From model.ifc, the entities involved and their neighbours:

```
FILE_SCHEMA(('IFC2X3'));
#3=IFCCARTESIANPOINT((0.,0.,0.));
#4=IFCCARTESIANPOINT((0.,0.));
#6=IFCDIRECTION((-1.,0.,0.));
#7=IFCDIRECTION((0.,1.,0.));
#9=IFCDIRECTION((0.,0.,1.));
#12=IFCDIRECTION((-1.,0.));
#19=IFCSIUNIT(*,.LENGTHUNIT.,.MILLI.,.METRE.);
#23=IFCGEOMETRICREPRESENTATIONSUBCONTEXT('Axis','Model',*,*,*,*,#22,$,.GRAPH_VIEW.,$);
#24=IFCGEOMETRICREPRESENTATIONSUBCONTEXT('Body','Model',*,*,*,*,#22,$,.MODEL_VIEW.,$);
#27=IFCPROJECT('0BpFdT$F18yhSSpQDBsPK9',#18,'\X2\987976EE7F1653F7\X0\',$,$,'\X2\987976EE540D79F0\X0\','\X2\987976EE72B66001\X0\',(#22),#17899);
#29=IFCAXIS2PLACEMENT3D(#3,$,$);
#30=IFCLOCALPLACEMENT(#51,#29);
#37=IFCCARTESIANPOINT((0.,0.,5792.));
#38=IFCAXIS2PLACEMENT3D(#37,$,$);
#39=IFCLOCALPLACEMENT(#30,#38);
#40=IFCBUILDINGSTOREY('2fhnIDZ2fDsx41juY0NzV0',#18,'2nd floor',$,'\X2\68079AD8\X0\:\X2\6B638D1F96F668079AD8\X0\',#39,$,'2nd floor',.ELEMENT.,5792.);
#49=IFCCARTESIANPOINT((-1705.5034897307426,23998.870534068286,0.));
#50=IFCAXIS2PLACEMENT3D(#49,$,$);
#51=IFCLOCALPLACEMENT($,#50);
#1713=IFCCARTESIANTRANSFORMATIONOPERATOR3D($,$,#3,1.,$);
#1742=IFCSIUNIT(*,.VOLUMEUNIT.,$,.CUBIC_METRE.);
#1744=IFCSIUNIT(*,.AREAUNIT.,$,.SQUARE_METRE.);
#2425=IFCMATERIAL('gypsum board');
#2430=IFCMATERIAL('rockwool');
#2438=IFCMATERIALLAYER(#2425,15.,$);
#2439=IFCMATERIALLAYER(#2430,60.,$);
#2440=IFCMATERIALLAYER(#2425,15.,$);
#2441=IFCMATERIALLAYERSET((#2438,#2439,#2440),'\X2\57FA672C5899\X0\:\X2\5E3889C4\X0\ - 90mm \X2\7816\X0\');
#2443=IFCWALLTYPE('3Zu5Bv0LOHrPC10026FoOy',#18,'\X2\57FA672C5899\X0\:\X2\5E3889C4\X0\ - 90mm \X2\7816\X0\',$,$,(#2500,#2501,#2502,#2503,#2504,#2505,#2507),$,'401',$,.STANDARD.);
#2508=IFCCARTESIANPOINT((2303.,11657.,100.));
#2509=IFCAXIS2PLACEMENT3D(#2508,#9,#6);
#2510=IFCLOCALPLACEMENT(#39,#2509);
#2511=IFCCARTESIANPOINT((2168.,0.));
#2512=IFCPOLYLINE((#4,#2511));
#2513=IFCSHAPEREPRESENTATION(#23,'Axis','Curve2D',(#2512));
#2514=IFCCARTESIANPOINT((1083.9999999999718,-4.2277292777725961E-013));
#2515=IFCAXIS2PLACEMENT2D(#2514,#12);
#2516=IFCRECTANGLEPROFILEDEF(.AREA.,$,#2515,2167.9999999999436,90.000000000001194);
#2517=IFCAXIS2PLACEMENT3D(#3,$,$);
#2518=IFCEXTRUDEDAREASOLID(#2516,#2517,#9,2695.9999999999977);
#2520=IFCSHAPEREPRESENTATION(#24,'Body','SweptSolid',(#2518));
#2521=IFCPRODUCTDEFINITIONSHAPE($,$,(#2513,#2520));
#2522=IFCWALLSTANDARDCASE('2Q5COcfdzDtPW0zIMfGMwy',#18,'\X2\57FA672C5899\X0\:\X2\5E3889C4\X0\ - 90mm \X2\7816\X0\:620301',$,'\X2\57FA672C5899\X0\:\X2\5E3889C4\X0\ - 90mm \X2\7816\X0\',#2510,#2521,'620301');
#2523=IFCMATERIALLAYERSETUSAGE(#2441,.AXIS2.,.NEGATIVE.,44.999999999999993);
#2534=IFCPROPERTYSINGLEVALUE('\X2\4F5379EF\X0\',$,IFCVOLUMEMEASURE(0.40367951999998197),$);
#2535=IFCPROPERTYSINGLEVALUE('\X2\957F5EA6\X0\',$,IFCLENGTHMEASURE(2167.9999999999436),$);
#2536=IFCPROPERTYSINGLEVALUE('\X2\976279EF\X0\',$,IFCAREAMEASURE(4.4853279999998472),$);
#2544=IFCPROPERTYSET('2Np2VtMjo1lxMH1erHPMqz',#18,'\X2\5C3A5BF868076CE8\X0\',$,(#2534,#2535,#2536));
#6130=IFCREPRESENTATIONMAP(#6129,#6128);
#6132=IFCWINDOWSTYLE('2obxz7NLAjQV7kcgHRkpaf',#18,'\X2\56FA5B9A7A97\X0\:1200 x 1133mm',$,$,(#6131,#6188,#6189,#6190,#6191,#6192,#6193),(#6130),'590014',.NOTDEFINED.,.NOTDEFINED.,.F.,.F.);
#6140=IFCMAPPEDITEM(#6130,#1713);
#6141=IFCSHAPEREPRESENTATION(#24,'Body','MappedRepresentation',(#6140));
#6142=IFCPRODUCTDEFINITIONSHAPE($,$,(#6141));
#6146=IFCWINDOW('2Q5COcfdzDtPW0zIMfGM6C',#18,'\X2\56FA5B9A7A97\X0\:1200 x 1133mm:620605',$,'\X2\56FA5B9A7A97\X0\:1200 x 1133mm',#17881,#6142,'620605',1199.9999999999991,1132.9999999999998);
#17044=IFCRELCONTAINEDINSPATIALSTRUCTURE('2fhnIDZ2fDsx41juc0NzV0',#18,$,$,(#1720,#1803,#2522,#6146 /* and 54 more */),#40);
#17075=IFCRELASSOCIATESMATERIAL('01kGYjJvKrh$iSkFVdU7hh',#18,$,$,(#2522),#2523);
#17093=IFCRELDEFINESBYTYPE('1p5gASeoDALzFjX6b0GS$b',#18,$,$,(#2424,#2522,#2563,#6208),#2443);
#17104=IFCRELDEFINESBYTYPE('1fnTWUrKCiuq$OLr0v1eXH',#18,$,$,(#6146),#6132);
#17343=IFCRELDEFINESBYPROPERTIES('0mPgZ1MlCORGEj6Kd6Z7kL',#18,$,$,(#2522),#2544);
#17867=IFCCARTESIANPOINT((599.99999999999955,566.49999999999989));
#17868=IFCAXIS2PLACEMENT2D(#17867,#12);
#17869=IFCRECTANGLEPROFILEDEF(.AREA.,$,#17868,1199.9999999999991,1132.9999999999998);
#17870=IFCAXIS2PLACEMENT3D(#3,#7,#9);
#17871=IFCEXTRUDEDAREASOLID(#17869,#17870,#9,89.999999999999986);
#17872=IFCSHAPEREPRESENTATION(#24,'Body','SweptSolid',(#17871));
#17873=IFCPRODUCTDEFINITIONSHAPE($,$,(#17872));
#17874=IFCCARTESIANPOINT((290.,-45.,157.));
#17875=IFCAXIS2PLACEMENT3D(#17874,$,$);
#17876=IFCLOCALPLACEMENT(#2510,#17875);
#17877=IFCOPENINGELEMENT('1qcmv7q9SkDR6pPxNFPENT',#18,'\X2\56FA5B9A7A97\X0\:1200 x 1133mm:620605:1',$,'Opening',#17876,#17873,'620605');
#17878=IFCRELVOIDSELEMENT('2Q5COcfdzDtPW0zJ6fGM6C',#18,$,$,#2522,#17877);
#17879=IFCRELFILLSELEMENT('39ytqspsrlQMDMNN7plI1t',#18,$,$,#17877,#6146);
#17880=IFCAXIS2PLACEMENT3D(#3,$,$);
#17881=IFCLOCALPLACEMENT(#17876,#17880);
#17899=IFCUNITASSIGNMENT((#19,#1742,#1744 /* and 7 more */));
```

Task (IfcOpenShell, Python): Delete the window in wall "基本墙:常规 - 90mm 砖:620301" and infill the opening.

```python
import ifcopenshell
import ifcopenshell.api.feature
import ifcopenshell.api.pset
import ifcopenshell.api.root
import ifcopenshell.geom
import ifcopenshell.util.element
import ifcopenshell.util.shape
import ifcopenshell.util.unit

model = ifcopenshell.open("model.ifc")
area_scale = ifcopenshell.util.unit.calculate_unit_scale(model, "AREAUNIT")
volume_scale = ifcopenshell.util.unit.calculate_unit_scale(model, "VOLUMEUNIT")
settings = ifcopenshell.geom.settings()


def volume(element):
    """Net volume in cubic metres, openings subtracted."""
    shape = ifcopenshell.geom.create_shape(settings, element)
    return ifcopenshell.util.shape.get_volume(shape.geometry)


window = model.by_id(6146)
opening = window.FillsVoids[0].RelatingOpeningElement
wall = opening.VoidsElements[0].RelatingBuildingElement
before = volume(wall)

ifcopenshell.api.root.remove_product(model, product=window)
ifcopenshell.api.feature.remove_feature(model, feature=opening)

after = volume(wall)
thickness = 0.09  # wall thickness in metres

# Update the wall's stored quantities.
pset = model.by_id(ifcopenshell.util.element.get_pset(wall, "尺寸标注", should_inherit=False)["id"])
ifcopenshell.api.pset.edit_pset(model, pset=pset, properties={
    "体积": model.create_entity("IfcVolumeMeasure", after / volume_scale),
    "面积": model.create_entity("IfcAreaMeasure", after / thickness / area_scale),
})

print(f"wall volume {before:.3f} -> {after:.3f} m3")

model.write("model_updated.ifc")
```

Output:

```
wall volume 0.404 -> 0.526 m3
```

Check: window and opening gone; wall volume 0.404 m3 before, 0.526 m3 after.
